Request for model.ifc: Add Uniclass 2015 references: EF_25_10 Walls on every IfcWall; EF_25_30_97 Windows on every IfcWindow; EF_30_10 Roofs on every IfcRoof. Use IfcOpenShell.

First a look at what the model holds.

```python
import ifcopenshell

model = ifcopenshell.open("model.ifc")
print(model.schema)
print("classifications:", [c.Name for c in model.by_type("IfcClassification")])
for ifc_class in ("IfcDoor", "IfcRoof", "IfcStair", "IfcWall", "IfcWindow"):
    print(ifc_class, len(model.by_type(ifc_class)))
```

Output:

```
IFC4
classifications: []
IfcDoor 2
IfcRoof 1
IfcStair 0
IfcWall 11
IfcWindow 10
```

```python
import ifcopenshell
import ifcopenshell.api.classification

model = ifcopenshell.open("model.ifc")

system = ifcopenshell.api.classification.add_classification(model, classification="Uniclass 2015")

codes = {
    "IfcWall": ("EF_25_10", "Walls"),
    "IfcWindow": ("EF_25_30_97", "Windows"),
    "IfcRoof": ("EF_30_10", "Roofs"),
}
for ifc_class, (code, name) in codes.items():
    products = model.by_type(ifc_class)
    ifcopenshell.api.classification.add_reference(
        model, products=products, classification=system, identification=code, name=name
    )
    print(code, len(products))

model.write("model_updated.ifc")
```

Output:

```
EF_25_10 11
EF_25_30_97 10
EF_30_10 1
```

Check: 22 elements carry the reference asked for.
